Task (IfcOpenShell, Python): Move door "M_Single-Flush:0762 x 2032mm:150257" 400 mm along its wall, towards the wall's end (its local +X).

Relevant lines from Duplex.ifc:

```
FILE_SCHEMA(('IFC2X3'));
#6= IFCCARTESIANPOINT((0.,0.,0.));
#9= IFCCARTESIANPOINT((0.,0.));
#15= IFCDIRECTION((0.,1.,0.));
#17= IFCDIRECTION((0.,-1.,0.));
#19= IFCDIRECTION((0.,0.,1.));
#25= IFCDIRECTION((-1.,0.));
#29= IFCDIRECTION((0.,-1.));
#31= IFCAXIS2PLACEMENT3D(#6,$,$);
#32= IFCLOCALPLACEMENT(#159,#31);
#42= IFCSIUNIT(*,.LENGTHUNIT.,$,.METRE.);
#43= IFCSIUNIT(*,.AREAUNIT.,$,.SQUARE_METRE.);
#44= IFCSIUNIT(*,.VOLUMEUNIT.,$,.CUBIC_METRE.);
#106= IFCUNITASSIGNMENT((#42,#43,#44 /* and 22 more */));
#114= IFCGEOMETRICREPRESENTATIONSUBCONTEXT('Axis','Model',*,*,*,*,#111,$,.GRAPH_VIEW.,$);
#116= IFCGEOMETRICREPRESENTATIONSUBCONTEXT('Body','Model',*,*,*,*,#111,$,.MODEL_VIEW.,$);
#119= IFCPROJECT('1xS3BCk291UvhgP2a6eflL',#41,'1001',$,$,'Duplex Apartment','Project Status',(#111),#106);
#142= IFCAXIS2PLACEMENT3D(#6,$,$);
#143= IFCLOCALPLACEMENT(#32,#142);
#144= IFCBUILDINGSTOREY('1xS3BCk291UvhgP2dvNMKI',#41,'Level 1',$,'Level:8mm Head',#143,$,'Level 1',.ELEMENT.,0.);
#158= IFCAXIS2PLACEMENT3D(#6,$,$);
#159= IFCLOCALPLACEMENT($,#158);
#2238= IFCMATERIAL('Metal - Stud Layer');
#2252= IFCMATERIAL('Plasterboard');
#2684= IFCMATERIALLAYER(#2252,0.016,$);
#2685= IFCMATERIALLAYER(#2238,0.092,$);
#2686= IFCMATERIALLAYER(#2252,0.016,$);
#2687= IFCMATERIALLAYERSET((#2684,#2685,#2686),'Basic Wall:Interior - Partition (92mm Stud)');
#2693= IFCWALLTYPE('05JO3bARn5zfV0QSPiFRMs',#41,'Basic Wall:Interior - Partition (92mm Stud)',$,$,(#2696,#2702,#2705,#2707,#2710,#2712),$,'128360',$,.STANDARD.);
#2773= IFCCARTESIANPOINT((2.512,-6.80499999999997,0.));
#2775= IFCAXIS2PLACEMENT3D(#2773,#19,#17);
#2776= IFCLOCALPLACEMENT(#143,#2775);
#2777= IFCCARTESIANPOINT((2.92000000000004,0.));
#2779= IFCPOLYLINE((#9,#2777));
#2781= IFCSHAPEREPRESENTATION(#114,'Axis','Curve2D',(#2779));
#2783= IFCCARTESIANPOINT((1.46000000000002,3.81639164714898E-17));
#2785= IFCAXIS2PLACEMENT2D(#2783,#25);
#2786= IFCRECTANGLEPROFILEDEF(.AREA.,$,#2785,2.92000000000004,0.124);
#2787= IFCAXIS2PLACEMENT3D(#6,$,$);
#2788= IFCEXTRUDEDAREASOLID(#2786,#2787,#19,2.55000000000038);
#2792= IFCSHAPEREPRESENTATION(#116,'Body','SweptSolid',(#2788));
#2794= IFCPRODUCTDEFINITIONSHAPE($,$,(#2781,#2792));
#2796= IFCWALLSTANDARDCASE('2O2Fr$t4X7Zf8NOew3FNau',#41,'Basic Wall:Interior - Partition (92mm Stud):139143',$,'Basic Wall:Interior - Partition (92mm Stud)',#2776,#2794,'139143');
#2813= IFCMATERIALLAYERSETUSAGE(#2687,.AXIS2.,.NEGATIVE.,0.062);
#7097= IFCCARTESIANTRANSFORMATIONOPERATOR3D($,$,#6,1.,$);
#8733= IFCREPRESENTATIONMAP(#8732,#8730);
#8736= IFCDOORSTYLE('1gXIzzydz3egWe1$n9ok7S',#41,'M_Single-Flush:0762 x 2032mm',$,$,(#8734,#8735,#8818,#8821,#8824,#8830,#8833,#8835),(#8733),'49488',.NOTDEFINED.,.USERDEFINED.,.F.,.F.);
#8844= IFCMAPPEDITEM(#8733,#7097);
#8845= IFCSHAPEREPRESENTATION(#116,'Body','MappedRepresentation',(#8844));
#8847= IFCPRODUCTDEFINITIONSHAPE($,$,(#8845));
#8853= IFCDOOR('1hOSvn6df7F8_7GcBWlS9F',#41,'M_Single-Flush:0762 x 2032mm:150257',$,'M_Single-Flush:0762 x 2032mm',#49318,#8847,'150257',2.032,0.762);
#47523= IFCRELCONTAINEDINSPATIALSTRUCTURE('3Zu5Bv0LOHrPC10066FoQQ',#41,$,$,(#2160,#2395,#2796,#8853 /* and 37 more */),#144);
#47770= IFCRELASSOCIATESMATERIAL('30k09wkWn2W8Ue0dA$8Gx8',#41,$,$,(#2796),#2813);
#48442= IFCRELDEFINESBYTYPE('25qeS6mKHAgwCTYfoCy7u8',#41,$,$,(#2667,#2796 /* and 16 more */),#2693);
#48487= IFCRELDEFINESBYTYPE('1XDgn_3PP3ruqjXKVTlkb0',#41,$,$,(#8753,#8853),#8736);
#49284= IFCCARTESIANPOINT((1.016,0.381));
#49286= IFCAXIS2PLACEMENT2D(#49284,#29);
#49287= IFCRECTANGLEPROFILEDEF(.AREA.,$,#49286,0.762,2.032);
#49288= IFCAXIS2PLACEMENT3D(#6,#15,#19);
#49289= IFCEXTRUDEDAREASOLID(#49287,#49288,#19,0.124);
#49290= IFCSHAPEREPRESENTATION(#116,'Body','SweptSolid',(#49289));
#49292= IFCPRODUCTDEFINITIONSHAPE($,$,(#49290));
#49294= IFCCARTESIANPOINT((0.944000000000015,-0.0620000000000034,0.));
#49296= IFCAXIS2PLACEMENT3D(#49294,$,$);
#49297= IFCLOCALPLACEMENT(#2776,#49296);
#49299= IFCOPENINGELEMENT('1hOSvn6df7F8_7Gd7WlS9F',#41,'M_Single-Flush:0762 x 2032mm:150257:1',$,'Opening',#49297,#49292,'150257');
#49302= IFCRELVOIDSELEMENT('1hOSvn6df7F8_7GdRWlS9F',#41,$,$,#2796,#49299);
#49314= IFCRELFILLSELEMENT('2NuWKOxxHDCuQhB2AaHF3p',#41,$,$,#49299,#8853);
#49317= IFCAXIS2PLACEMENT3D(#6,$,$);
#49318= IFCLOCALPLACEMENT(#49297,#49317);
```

```python
import ifcopenshell
import ifcopenshell.api.geometry
import ifcopenshell.util.placement

model = ifcopenshell.open("Duplex.ifc")

door = model.by_id(8853)
opening = door.FillsVoids[0].RelatingOpeningElement
wall = opening.VoidsElements[0].RelatingBuildingElement

wall_matrix = ifcopenshell.util.placement.get_local_placement(wall.ObjectPlacement)
shift = wall_matrix[:3, 0] * 0.4
before = ifcopenshell.util.placement.get_local_placement(door.ObjectPlacement)[:3, 3].copy()

# The door is placed relative to its opening, so it follows when the opening moves.
matrix = ifcopenshell.util.placement.get_local_placement(opening.ObjectPlacement)
matrix[:3, 3] += shift
ifcopenshell.api.geometry.edit_object_placement(
    model, product=opening, matrix=matrix, is_si=False, should_transform_children=True
)

after = ifcopenshell.util.placement.get_local_placement(door.ObjectPlacement)[:3, 3]
print("door moved by", (after - before).round(3) + 0.0)

model.write("Duplex_v2.ifc")
```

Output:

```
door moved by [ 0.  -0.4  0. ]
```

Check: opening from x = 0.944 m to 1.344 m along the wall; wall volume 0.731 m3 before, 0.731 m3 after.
